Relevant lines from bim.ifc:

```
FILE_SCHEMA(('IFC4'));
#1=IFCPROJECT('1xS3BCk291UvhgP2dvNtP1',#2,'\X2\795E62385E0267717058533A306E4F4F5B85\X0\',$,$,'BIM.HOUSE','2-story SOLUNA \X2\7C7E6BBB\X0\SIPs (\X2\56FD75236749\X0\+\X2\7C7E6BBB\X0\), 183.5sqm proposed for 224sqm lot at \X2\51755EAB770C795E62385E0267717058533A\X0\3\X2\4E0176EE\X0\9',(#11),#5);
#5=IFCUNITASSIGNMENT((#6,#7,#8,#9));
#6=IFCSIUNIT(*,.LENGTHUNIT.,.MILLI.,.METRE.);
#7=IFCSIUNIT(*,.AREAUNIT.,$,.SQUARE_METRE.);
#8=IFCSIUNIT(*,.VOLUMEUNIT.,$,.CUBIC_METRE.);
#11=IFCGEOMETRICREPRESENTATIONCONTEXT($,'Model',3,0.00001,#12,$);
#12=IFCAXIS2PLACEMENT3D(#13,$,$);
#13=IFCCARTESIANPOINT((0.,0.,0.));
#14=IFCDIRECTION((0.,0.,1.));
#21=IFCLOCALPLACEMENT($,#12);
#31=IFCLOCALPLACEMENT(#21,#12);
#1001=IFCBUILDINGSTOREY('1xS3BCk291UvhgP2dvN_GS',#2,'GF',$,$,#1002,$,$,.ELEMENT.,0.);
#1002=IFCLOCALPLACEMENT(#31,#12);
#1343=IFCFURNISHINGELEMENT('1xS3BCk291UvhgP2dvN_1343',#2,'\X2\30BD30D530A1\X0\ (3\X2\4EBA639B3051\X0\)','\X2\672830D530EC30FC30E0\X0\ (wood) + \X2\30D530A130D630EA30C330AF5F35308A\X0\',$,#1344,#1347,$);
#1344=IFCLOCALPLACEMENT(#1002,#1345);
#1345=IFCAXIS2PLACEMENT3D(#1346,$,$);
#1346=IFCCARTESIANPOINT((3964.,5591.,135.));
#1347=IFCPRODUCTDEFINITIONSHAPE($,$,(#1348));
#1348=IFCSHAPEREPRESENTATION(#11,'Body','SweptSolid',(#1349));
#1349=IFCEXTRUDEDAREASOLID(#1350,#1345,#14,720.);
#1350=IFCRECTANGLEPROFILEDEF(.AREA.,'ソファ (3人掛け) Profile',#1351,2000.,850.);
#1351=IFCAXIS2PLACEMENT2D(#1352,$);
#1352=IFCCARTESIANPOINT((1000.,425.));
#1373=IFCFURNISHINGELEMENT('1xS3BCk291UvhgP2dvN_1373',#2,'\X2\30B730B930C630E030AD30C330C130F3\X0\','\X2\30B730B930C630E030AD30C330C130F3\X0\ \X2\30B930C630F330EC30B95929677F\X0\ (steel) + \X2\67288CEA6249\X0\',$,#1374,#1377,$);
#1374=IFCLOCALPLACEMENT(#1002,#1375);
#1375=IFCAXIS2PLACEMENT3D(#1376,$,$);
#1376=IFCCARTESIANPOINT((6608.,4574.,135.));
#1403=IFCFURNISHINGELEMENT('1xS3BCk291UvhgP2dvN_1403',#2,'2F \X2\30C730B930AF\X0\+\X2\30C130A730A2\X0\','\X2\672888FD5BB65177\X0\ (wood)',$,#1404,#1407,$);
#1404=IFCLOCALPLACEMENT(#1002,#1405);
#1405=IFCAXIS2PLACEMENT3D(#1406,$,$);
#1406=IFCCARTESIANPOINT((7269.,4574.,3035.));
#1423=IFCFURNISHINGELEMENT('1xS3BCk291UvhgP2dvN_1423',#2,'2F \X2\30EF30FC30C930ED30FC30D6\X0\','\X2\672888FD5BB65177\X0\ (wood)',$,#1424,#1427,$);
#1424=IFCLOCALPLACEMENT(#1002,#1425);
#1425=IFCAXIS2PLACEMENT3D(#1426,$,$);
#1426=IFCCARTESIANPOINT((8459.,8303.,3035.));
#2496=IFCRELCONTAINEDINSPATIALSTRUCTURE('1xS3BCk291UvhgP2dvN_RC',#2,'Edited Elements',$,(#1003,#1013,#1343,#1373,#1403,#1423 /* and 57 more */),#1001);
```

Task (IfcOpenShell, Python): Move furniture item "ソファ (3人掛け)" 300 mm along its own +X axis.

```python
import ifcopenshell
import ifcopenshell.api.geometry
import ifcopenshell.util.placement
import ifcopenshell.util.unit

model = ifcopenshell.open("bim.ifc")
unit_scale = ifcopenshell.util.unit.calculate_unit_scale(model)

item = model.by_id(1343)
matrix = ifcopenshell.util.placement.get_local_placement(item.ObjectPlacement)
matrix[:3, 3] += matrix[:3, 0] * 0.3 / unit_scale
ifcopenshell.api.geometry.edit_object_placement(model, product=item, matrix=matrix, is_si=False)

print(ifcopenshell.util.placement.get_local_placement(item.ObjectPlacement).round(3) + 0.0)

model.write("bim_rev.ifc")
```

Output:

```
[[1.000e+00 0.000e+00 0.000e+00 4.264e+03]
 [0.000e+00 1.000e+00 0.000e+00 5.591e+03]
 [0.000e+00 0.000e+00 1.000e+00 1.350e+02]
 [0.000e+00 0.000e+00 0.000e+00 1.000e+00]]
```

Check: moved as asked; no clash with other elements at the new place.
